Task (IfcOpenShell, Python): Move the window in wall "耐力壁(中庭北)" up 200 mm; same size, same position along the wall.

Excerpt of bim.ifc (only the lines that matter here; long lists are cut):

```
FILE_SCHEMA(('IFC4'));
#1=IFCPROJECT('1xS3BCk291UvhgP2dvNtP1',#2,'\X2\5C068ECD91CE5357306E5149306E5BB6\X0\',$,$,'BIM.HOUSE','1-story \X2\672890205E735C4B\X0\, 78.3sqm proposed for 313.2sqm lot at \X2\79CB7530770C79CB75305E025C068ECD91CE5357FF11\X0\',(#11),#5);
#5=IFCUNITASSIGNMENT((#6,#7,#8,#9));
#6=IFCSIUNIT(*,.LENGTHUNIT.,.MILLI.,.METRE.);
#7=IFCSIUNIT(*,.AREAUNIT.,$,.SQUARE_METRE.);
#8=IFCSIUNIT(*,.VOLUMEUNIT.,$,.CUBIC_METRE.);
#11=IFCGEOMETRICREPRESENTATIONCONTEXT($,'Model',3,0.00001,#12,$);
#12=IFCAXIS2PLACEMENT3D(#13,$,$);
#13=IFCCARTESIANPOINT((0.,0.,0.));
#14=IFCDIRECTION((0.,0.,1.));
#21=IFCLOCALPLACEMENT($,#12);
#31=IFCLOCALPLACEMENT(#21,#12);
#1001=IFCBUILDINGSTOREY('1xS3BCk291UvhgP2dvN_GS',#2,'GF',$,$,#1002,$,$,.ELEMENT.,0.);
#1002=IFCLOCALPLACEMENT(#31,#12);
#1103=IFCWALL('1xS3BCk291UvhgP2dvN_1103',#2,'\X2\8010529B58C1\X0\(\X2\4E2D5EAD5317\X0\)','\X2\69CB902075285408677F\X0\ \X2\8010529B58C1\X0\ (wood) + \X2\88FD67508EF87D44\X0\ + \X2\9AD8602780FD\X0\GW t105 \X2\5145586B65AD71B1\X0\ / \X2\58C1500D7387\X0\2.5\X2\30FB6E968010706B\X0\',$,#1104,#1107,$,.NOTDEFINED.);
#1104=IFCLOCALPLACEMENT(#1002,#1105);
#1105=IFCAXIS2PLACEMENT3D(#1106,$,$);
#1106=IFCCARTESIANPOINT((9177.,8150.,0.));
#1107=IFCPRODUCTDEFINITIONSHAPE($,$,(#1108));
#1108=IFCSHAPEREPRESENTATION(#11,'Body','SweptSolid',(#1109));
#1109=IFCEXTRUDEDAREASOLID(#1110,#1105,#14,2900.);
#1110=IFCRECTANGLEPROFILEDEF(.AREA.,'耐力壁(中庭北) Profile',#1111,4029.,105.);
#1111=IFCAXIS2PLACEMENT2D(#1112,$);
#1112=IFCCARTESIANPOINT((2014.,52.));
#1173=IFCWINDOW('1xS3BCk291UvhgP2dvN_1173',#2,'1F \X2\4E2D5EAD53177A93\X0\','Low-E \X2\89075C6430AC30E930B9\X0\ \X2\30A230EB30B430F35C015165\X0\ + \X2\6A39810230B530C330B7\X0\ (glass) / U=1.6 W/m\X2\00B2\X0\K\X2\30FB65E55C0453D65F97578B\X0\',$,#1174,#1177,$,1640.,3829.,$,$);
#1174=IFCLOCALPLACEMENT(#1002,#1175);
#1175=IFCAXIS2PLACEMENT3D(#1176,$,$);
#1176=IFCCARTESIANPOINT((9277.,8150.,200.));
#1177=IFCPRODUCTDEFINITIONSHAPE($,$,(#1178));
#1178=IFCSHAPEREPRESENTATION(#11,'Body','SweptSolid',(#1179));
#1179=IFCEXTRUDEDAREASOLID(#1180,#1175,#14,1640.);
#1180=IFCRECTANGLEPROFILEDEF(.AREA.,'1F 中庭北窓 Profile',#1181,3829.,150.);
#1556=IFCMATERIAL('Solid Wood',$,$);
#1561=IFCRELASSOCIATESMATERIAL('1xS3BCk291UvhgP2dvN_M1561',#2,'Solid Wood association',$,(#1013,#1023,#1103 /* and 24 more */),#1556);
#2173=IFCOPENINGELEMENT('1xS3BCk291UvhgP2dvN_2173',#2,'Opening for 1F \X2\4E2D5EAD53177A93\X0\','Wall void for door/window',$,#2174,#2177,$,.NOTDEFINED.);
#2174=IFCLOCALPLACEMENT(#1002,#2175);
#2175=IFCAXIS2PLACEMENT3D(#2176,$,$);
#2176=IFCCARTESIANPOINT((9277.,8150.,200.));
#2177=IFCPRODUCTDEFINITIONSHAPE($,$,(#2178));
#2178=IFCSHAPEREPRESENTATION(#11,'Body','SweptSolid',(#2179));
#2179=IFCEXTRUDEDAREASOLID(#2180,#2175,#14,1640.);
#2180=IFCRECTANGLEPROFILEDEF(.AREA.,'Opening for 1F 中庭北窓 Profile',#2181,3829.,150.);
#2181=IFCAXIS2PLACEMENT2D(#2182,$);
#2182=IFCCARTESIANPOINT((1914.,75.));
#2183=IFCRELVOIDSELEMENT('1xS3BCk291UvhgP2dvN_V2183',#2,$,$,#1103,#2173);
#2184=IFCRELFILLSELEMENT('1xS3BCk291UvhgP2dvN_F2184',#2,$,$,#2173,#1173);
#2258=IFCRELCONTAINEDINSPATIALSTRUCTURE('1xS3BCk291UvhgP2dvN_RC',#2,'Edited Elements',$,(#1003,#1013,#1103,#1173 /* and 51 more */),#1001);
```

```python
import numpy as np
import ifcopenshell
import ifcopenshell.api.geometry
import ifcopenshell.util.placement
import ifcopenshell.util.unit

model = ifcopenshell.open("bim.ifc")
unit_scale = ifcopenshell.util.unit.calculate_unit_scale(model)

window = model.by_guid("1xS3BCk291UvhgP2dvN_1173")
opening = window.FillsVoids[0].RelatingOpeningElement
dz = 200.0

shift = np.array([0.0, 0.0, dz])
# The window is not placed relative to its opening, so move both.
for product in (opening, window):
    matrix = ifcopenshell.util.placement.get_local_placement(product.ObjectPlacement)
    matrix[:3, 3] += shift
    ifcopenshell.api.geometry.edit_object_placement(model, product=product, matrix=matrix, is_si=False)

print(f"moved by {dz * unit_scale:+.3f} m")

model.write("bim_v2.ifc")
```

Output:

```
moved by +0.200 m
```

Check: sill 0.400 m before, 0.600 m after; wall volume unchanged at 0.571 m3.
